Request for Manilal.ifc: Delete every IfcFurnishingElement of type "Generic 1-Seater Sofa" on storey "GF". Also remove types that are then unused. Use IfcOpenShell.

First a look at what the model holds.

```python
import ifcopenshell
import ifcopenshell.util.element

model = ifcopenshell.open("Manilal.ifc")
print(model.schema)
storey = next(s for s in model.by_type("IfcBuildingStorey") if s.Name == "GF")
furniture = [e for e in ifcopenshell.util.element.get_decomposition(storey) if e.is_a("IfcFurnishingElement")]
seen = {}
for e in furniture:
    element_type = ifcopenshell.util.element.get_type(e)
    name = element_type.Name if element_type not in (None, e) else None
    seen[name] = seen.get(name, 0) + 1
for name, count in sorted(seen.items(), key=str):
    print(count, "x", name)
```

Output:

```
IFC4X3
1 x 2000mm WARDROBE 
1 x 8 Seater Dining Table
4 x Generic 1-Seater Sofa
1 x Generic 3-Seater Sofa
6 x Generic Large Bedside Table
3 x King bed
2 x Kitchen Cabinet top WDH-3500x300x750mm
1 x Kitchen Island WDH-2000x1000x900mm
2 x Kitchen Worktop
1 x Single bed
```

```python
import ifcopenshell
import ifcopenshell.api.root
import ifcopenshell.util.element

model = ifcopenshell.open("Manilal.ifc")

storey = next(s for s in model.by_type("IfcBuildingStorey") if s.Name == "GF")
furniture = [e for e in ifcopenshell.util.element.get_decomposition(storey) if e.is_a("IfcFurnishingElement")]
targets = [e for e in furniture if (t := ifcopenshell.util.element.get_type(e)) not in (None, e) and t.Name == "Generic 1-Seater Sofa"]
types = {ifcopenshell.util.element.get_type(e) for e in targets} - {None, *targets}

for e in targets:
    ifcopenshell.api.root.remove_product(model, product=e)
print(len(targets), "removed")

unused = [t for t in types if not ifcopenshell.util.element.get_types(t)]
for t in unused:
    ifcopenshell.api.root.remove_product(model, product=t)
print(len(unused), "unused types removed")

model.write("Manilal_updated.ifc")
```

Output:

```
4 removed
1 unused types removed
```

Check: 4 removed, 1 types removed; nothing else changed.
